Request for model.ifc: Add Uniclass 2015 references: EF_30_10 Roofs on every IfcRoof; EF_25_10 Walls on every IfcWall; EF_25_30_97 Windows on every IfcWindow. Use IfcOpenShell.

First a look at what the model holds.

```python
import ifcopenshell

model = ifcopenshell.open("model.ifc")
print(model.schema)
print("classifications:", [c.Name for c in model.by_type("IfcClassification")])
for ifc_class in ("IfcDoor", "IfcRoof", "IfcStair", "IfcWall", "IfcWindow"):
    print(ifc_class, len(model.by_type(ifc_class)))
```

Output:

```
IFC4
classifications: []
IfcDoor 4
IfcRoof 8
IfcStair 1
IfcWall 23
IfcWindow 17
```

```python
import ifcopenshell
import ifcopenshell.api.classification

model = ifcopenshell.open("model.ifc")

system = ifcopenshell.api.classification.add_classification(model, classification="Uniclass 2015")

codes = {
    "IfcRoof": ("EF_30_10", "Roofs"),
    "IfcWall": ("EF_25_10", "Walls"),
    "IfcWindow": ("EF_25_30_97", "Windows"),
}
for ifc_class, (code, name) in codes.items():
    products = model.by_type(ifc_class)
    ifcopenshell.api.classification.add_reference(
        model, products=products, classification=system, identification=code, name=name
    )
    print(code, len(products))

model.write("model-out.ifc")
```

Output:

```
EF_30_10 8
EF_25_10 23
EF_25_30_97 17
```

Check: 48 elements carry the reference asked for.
